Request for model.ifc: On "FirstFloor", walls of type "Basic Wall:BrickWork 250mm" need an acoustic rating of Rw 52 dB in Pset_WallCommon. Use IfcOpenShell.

First a look at what the model holds.

```python
import ifcopenshell
import ifcopenshell.util.element

model = ifcopenshell.open("model.ifc")
print(model.schema)
storey = next(s for s in model.by_type("IfcBuildingStorey") if s.Name == "FirstFloor")
walls = [e for e in ifcopenshell.util.element.get_decomposition(storey) if e.is_a("IfcWall")]
seen = {}
for e in walls:
    element_type = ifcopenshell.util.element.get_type(e)
    key = (element_type.Name if element_type != e and element_type else None, ifcopenshell.util.element.get_pset(e, "Pset_WallCommon", "AcousticRating"))
    seen[key] = seen.get(key, 0) + 1
for (name, value), count in sorted(seen.items(), key=str):
    print(count, "x", name, "|", value)
```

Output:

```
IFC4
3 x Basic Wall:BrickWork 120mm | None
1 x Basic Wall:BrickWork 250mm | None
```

```python
import ifcopenshell
import ifcopenshell.api.pset
import ifcopenshell.util.element

model = ifcopenshell.open("model.ifc")

storey = next(s for s in model.by_type("IfcBuildingStorey") if s.Name == "FirstFloor")
walls = [e for e in ifcopenshell.util.element.get_decomposition(storey) if e.is_a("IfcWall")]

count = 0
for e in walls:
    element_type = ifcopenshell.util.element.get_type(e)
    if element_type in (None, e) or element_type.Name != "Basic Wall:BrickWork 250mm":
        continue
    # add_pset returns the element's existing set when there is one.
    pset = ifcopenshell.api.pset.add_pset(model, product=e, name="Pset_WallCommon")
    ifcopenshell.api.pset.edit_pset(model, pset=pset, properties={"AcousticRating": "Rw 52 dB"})
    count += 1

print(count, "walls updated")

model.write("model_updated.ifc")
```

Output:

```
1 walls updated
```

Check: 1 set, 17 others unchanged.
